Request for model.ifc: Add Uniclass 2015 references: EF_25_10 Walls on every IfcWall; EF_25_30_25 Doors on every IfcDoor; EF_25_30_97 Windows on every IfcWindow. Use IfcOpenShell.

First a look at what the model holds.

```python
import ifcopenshell

model = ifcopenshell.open("model.ifc")
print(model.schema)
print("classifications:", [c.Name for c in model.by_type("IfcClassification")])
for ifc_class in ("IfcDoor", "IfcRoof", "IfcStair", "IfcWall", "IfcWindow"):
    print(ifc_class, len(model.by_type(ifc_class)))
```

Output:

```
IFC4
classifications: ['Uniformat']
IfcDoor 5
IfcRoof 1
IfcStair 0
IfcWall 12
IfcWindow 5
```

```python
import ifcopenshell
import ifcopenshell.api.classification

model = ifcopenshell.open("model.ifc")

system = ifcopenshell.api.classification.add_classification(model, classification="Uniclass 2015")

codes = {
    "IfcWall": ("EF_25_10", "Walls"),
    "IfcDoor": ("EF_25_30_25", "Doors"),
    "IfcWindow": ("EF_25_30_97", "Windows"),
}
for ifc_class, (code, name) in codes.items():
    products = model.by_type(ifc_class)
    ifcopenshell.api.classification.add_reference(
        model, products=products, classification=system, identification=code, name=name
    )
    print(code, len(products))

model.write("model_edited.ifc")
```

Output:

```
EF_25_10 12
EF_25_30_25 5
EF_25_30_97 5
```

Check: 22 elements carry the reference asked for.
